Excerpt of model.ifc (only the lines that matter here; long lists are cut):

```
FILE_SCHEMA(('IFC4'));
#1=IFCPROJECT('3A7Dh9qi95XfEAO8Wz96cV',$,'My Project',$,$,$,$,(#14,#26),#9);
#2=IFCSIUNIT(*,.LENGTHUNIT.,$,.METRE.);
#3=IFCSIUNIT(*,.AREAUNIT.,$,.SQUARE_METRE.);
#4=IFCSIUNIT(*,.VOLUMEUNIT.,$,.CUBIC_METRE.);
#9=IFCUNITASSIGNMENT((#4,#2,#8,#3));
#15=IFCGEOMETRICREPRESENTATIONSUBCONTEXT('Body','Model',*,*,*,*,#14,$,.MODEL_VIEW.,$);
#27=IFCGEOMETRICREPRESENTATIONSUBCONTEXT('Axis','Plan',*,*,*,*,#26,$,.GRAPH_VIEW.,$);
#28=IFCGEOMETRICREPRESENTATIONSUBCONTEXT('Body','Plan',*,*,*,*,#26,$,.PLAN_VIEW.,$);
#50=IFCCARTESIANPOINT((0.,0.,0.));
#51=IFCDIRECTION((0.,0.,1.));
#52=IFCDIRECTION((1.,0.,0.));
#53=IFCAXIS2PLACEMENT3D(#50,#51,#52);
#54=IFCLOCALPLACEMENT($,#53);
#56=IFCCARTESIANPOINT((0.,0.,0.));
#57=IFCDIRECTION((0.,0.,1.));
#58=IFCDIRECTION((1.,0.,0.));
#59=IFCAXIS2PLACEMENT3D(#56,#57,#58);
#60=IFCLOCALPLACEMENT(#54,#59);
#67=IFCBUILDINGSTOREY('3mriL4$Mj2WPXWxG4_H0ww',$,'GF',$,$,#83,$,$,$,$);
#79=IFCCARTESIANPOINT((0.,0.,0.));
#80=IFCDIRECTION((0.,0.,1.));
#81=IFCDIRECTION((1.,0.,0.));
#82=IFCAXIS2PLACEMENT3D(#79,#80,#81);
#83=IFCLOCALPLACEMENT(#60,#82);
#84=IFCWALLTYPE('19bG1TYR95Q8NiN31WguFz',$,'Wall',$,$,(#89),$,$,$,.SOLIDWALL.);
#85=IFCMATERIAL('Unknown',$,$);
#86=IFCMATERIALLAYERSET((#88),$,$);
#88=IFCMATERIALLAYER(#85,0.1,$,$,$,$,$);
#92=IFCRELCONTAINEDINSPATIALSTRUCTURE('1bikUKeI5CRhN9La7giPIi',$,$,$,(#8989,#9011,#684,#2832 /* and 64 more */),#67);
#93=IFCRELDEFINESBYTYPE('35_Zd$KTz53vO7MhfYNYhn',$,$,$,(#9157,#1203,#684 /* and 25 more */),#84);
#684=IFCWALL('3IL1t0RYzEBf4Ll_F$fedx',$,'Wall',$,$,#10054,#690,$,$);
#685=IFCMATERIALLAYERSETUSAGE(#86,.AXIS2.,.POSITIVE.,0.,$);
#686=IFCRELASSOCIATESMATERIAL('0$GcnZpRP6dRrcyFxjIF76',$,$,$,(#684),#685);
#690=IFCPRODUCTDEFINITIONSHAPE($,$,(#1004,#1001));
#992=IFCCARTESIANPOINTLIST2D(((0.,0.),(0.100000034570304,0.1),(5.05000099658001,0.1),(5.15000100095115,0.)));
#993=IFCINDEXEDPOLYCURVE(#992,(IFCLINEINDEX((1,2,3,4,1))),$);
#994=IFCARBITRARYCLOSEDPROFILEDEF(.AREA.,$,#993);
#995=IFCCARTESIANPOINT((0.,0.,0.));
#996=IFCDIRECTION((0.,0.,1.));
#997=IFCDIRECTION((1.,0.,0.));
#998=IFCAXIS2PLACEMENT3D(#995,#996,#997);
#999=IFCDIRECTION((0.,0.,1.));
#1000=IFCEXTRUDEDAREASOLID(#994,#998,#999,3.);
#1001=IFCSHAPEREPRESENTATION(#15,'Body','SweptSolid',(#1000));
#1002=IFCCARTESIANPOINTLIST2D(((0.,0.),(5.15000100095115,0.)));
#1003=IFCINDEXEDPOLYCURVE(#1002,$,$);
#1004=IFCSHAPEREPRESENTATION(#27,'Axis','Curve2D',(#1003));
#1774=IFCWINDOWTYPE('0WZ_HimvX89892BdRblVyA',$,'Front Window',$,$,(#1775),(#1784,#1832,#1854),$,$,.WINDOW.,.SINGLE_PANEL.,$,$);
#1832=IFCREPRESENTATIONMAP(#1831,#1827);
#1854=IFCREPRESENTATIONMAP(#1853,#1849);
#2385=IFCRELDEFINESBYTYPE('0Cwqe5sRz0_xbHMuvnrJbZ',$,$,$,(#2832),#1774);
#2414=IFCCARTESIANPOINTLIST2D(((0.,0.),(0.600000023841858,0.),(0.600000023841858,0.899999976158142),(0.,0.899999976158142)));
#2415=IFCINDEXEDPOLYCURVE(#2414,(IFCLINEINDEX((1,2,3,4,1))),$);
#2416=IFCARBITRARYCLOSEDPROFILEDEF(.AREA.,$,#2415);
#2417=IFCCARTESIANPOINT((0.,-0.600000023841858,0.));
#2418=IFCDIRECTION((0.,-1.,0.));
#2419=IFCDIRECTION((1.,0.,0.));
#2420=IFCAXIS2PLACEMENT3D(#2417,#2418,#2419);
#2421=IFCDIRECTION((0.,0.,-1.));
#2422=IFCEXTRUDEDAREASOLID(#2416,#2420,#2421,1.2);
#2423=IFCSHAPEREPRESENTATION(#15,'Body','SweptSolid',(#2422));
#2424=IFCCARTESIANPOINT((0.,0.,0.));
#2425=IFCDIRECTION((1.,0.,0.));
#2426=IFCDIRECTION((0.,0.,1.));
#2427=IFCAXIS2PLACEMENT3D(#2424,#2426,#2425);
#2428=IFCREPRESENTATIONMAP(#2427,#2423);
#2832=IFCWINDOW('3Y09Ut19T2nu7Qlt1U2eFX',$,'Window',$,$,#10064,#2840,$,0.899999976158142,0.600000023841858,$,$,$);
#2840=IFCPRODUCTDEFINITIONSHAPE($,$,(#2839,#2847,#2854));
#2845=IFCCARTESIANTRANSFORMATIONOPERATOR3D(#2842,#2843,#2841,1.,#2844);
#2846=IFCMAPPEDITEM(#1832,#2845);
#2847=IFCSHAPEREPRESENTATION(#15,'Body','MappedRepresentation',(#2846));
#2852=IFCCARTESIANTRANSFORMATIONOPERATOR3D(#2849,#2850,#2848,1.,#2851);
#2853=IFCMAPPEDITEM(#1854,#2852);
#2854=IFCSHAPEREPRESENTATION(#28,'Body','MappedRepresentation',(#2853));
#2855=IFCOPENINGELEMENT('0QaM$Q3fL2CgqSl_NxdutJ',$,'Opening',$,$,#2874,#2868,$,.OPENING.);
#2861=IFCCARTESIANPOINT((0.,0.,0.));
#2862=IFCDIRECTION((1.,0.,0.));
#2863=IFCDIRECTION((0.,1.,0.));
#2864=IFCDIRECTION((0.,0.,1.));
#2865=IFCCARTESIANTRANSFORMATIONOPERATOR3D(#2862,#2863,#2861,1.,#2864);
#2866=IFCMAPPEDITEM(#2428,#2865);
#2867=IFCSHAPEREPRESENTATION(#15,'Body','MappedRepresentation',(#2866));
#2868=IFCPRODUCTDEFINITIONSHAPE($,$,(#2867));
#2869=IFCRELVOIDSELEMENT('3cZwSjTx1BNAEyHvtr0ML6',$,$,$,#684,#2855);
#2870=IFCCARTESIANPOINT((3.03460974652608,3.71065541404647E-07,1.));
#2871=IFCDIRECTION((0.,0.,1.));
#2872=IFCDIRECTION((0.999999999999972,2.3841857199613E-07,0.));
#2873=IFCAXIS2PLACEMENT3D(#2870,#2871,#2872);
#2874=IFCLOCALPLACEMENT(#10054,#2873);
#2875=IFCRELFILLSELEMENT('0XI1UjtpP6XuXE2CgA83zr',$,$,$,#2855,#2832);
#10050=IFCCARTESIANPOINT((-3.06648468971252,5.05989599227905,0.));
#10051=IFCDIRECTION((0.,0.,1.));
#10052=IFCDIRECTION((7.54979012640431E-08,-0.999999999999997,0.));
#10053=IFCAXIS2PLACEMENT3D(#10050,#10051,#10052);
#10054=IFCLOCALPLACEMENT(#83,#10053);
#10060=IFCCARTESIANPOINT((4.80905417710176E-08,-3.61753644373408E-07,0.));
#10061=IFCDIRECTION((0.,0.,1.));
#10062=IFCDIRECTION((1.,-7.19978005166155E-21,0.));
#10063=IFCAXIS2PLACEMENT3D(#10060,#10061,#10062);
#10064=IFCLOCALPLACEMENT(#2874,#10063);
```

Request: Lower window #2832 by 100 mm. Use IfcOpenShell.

```python
import numpy as np
import ifcopenshell
import ifcopenshell.api.geometry
import ifcopenshell.util.placement
import ifcopenshell.util.unit

model = ifcopenshell.open("model.ifc")
unit_scale = ifcopenshell.util.unit.calculate_unit_scale(model)

window = model.by_guid("3Y09Ut19T2nu7Qlt1U2eFX")
opening = window.FillsVoids[0].RelatingOpeningElement
dz = -0.1 / unit_scale

shift = np.array([0.0, 0.0, dz])
# The window is placed relative to its opening, so it follows when the opening moves.
matrix = ifcopenshell.util.placement.get_local_placement(opening.ObjectPlacement)
matrix[:3, 3] += shift
ifcopenshell.api.geometry.edit_object_placement(
    model, product=opening, matrix=matrix, is_si=False, should_transform_children=True
)

print(f"moved by {dz * unit_scale:+.3f} m")

model.write("model_v2.ifc")
```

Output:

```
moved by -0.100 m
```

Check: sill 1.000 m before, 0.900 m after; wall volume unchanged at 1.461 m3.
